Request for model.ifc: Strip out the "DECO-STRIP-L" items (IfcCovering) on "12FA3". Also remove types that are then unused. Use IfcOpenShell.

First a look at what the model holds.

```python
import ifcopenshell
import ifcopenshell.util.element

model = ifcopenshell.open("model.ifc")
print(model.schema)
storey = next(s for s in model.by_type("IfcBuildingStorey") if s.Name == "12FA3")
coverings = [e for e in ifcopenshell.util.element.get_decomposition(storey) if e.is_a("IfcCovering")]
seen = {}
for e in coverings:
    element_type = ifcopenshell.util.element.get_type(e)
    name = element_type.Name if element_type not in (None, e) else None
    seen[name] = seen.get(name, 0) + 1
for name, count in sorted(seen.items(), key=str):
    print(count, "x", name)
```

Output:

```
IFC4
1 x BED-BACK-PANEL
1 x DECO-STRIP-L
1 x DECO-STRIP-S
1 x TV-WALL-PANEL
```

```python
import ifcopenshell
import ifcopenshell.api.root
import ifcopenshell.util.element

model = ifcopenshell.open("model.ifc")

storey = next(s for s in model.by_type("IfcBuildingStorey") if s.Name == "12FA3")
coverings = [e for e in ifcopenshell.util.element.get_decomposition(storey) if e.is_a("IfcCovering")]
targets = [e for e in coverings if (t := ifcopenshell.util.element.get_type(e)) not in (None, e) and t.Name == "DECO-STRIP-L"]
types = {ifcopenshell.util.element.get_type(e) for e in targets} - {None, *targets}

for e in targets:
    ifcopenshell.api.root.remove_product(model, product=e)
print(len(targets), "removed")

unused = [t for t in types if not ifcopenshell.util.element.get_types(t)]
for t in unused:
    ifcopenshell.api.root.remove_product(model, product=t)
print(len(unused), "unused types removed")

model.write("model_edited.ifc")
```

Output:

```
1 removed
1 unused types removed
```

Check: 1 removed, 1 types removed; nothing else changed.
